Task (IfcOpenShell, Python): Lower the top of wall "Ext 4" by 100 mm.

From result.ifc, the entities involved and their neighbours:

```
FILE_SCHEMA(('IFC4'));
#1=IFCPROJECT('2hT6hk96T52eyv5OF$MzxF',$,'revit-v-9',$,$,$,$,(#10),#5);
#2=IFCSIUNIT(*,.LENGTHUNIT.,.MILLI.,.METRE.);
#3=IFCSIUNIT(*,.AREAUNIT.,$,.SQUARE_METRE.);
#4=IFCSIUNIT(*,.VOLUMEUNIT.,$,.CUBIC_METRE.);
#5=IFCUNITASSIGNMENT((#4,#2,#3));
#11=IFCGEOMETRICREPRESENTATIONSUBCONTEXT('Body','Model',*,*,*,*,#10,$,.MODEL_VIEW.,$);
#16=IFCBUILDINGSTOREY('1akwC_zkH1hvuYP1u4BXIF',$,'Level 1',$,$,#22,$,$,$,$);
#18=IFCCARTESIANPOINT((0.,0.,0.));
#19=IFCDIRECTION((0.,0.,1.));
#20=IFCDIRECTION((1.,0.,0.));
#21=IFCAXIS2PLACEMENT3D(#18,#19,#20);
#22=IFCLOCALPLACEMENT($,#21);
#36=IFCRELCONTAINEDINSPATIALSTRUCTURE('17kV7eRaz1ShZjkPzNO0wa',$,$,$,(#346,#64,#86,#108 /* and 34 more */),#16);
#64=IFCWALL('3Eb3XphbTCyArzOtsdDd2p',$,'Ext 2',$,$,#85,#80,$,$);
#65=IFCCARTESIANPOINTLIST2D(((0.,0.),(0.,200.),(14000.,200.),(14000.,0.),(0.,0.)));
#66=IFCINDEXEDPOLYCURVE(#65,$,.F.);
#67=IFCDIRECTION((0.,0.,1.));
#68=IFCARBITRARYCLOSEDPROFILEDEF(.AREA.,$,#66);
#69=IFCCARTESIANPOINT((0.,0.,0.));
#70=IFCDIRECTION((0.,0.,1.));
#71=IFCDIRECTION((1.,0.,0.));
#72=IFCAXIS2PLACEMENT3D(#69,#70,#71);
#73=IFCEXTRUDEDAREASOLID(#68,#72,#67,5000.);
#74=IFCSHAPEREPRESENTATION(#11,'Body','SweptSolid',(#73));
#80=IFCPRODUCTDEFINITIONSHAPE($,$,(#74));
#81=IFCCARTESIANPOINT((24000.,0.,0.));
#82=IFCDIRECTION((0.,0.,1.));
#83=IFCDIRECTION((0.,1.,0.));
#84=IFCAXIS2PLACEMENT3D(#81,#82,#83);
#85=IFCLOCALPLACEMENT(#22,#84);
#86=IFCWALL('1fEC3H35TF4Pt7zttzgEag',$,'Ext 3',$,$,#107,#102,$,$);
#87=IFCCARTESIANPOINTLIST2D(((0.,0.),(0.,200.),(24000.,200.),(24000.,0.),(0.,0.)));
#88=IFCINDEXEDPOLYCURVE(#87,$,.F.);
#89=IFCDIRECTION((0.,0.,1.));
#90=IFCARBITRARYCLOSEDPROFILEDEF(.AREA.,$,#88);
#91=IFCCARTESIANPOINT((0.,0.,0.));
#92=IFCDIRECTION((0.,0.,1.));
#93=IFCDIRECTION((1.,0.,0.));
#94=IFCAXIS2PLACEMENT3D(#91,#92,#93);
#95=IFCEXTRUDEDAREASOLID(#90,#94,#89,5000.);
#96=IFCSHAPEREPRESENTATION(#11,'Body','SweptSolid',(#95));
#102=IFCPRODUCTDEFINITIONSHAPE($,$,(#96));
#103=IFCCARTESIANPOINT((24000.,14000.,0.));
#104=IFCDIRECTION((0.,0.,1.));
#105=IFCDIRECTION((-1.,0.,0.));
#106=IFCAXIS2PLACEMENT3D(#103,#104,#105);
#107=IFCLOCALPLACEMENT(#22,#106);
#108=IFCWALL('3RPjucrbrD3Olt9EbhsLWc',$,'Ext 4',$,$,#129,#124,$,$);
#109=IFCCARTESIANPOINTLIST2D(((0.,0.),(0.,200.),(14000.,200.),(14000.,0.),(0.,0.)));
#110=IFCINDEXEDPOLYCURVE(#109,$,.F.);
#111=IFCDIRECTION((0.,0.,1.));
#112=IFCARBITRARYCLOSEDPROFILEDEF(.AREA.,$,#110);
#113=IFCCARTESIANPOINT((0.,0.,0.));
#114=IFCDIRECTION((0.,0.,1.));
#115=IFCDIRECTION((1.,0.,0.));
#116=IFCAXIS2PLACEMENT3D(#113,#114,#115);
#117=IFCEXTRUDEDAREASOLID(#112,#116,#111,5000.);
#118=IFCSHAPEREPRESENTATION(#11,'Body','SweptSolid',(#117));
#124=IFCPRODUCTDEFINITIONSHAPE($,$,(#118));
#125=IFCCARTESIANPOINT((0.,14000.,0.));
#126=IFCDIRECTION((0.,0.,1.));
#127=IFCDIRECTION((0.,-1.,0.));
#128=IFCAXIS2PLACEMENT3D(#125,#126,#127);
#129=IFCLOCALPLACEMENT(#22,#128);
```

```python
import ifcopenshell
import ifcopenshell.geom
import ifcopenshell.util.representation
import ifcopenshell.util.shape
import ifcopenshell.util.unit

model = ifcopenshell.open("result.ifc")
unit_scale = ifcopenshell.util.unit.calculate_unit_scale(model)
settings = ifcopenshell.geom.settings()


def volume(element):
    """Net volume in cubic metres, openings subtracted."""
    shape = ifcopenshell.geom.create_shape(settings, element)
    return ifcopenshell.util.shape.get_volume(shape.geometry)


wall = model.by_guid("3RPjucrbrD3Olt9EbhsLWc")
before = volume(wall)

body = ifcopenshell.util.representation.get_representation(wall, "Model", "Body")
solid = body.Items[0]
old_height = solid.Depth
solid.Depth -= 0.1 / unit_scale
after = volume(wall)

print(f"height {old_height:g} -> {solid.Depth:g}, volume {before:.3f} -> {after:.3f} m3")

model.write("result_v2.ifc")
```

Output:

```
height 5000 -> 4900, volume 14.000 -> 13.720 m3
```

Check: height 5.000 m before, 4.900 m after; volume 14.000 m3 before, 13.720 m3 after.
